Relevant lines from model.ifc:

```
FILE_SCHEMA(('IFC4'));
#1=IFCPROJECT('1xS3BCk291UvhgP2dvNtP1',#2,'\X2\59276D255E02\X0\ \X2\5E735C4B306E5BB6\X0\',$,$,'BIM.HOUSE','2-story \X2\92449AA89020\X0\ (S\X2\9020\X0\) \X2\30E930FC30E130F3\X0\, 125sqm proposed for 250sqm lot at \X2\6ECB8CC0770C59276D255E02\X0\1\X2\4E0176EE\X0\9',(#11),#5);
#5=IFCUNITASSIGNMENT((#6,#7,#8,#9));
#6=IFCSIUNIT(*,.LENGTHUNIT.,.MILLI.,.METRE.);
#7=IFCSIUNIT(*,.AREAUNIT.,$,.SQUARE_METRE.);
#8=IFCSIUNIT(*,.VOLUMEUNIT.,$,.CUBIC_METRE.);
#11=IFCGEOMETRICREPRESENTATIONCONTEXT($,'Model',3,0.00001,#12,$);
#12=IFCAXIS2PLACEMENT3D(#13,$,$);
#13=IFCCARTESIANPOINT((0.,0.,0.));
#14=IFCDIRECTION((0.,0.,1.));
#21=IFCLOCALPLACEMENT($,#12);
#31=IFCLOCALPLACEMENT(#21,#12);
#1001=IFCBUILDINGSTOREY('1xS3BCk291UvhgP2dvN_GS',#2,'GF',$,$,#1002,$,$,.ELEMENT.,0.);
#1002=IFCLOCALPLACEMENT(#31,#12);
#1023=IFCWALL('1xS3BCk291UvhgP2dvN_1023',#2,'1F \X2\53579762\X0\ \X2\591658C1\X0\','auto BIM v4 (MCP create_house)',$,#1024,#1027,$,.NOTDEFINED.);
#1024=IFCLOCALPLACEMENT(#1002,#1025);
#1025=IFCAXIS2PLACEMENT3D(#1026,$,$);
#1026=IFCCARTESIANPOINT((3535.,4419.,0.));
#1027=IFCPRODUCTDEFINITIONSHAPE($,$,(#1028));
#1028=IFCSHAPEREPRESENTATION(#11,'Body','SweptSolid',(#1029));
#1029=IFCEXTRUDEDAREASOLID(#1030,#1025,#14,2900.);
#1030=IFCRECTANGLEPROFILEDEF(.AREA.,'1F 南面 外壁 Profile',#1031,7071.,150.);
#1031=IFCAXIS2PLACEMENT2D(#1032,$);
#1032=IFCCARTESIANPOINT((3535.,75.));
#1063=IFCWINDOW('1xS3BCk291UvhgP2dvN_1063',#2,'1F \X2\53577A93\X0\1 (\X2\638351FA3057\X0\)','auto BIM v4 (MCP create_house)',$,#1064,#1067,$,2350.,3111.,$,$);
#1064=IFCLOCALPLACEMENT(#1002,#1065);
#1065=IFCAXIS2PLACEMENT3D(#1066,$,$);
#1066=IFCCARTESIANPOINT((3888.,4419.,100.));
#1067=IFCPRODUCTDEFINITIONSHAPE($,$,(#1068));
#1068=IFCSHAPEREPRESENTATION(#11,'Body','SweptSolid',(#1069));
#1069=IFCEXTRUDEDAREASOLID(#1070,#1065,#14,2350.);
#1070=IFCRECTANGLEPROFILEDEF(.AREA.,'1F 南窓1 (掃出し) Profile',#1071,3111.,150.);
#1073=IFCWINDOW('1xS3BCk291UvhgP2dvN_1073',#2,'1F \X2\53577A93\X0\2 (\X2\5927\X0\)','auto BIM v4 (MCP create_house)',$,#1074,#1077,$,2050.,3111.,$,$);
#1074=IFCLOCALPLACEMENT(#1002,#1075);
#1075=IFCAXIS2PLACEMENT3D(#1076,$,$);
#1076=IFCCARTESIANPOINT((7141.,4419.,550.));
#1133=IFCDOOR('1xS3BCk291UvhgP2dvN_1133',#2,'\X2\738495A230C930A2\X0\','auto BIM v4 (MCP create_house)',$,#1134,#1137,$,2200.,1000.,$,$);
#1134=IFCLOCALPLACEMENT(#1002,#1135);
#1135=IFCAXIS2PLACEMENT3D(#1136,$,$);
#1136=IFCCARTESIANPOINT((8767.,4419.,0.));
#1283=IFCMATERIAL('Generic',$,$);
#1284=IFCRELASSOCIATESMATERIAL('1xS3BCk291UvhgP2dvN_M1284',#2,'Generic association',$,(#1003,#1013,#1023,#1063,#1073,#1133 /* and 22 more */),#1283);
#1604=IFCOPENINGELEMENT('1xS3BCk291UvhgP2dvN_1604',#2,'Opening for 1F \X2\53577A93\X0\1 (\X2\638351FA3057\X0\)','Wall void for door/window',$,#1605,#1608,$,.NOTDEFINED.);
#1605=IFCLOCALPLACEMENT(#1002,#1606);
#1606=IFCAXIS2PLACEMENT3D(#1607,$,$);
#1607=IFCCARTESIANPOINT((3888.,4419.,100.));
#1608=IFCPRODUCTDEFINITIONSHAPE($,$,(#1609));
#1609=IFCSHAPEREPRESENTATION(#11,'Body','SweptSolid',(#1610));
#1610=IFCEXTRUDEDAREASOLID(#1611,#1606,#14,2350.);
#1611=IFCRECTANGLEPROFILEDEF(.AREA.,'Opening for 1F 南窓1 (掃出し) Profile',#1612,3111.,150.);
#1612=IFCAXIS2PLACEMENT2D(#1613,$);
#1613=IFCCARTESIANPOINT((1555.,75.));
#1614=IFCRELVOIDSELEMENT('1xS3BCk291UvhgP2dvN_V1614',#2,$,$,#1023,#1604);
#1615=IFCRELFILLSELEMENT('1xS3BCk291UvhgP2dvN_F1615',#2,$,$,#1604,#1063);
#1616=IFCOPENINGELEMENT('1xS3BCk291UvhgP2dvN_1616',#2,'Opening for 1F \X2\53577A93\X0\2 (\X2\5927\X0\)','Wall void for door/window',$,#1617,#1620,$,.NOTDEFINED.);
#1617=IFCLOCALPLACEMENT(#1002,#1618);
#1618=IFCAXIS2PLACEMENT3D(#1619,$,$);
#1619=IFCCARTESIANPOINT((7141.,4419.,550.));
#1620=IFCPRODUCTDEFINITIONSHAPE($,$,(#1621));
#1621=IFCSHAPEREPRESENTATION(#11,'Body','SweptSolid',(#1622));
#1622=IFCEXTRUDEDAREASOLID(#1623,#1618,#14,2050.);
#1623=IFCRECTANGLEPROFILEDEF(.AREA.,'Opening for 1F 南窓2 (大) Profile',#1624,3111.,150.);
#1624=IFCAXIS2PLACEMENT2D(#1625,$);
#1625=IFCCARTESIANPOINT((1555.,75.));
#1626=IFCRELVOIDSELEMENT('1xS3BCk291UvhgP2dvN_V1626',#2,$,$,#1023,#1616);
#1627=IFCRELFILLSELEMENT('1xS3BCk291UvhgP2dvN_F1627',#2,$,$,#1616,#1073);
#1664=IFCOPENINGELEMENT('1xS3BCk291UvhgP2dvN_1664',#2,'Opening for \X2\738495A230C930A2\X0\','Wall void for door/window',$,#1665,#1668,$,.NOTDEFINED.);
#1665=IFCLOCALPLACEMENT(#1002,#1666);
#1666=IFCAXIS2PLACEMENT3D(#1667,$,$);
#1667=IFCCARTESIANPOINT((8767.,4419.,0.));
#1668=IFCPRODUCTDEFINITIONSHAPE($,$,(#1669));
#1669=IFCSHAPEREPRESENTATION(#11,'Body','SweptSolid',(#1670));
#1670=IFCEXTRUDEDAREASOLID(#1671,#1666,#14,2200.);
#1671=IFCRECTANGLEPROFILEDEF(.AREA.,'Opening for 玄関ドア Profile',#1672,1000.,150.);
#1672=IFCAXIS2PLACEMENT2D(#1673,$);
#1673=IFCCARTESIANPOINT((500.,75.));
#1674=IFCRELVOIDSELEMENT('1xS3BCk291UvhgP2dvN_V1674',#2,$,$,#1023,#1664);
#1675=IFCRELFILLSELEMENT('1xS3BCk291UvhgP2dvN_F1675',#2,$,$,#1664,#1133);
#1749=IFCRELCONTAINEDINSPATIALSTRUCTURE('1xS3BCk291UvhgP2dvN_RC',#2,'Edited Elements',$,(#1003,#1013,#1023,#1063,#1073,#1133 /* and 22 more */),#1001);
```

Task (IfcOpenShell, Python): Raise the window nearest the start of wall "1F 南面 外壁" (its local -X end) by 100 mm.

```python
import numpy as np
import ifcopenshell
import ifcopenshell.api.geometry
import ifcopenshell.util.placement
import ifcopenshell.util.unit

model = ifcopenshell.open("model.ifc")
unit_scale = ifcopenshell.util.unit.calculate_unit_scale(model)

window = model.by_id(1063)
opening = window.FillsVoids[0].RelatingOpeningElement
dz = 100.0

shift = np.array([0.0, 0.0, dz])
# The window is not placed relative to its opening, so move both.
for product in (opening, window):
    matrix = ifcopenshell.util.placement.get_local_placement(product.ObjectPlacement)
    matrix[:3, 3] += shift
    ifcopenshell.api.geometry.edit_object_placement(model, product=product, matrix=matrix, is_si=False)

print(f"moved by {dz * unit_scale:+.3f} m")

model.write("model_edited.ifc")
```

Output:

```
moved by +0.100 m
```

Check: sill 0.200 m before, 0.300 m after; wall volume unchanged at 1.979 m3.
